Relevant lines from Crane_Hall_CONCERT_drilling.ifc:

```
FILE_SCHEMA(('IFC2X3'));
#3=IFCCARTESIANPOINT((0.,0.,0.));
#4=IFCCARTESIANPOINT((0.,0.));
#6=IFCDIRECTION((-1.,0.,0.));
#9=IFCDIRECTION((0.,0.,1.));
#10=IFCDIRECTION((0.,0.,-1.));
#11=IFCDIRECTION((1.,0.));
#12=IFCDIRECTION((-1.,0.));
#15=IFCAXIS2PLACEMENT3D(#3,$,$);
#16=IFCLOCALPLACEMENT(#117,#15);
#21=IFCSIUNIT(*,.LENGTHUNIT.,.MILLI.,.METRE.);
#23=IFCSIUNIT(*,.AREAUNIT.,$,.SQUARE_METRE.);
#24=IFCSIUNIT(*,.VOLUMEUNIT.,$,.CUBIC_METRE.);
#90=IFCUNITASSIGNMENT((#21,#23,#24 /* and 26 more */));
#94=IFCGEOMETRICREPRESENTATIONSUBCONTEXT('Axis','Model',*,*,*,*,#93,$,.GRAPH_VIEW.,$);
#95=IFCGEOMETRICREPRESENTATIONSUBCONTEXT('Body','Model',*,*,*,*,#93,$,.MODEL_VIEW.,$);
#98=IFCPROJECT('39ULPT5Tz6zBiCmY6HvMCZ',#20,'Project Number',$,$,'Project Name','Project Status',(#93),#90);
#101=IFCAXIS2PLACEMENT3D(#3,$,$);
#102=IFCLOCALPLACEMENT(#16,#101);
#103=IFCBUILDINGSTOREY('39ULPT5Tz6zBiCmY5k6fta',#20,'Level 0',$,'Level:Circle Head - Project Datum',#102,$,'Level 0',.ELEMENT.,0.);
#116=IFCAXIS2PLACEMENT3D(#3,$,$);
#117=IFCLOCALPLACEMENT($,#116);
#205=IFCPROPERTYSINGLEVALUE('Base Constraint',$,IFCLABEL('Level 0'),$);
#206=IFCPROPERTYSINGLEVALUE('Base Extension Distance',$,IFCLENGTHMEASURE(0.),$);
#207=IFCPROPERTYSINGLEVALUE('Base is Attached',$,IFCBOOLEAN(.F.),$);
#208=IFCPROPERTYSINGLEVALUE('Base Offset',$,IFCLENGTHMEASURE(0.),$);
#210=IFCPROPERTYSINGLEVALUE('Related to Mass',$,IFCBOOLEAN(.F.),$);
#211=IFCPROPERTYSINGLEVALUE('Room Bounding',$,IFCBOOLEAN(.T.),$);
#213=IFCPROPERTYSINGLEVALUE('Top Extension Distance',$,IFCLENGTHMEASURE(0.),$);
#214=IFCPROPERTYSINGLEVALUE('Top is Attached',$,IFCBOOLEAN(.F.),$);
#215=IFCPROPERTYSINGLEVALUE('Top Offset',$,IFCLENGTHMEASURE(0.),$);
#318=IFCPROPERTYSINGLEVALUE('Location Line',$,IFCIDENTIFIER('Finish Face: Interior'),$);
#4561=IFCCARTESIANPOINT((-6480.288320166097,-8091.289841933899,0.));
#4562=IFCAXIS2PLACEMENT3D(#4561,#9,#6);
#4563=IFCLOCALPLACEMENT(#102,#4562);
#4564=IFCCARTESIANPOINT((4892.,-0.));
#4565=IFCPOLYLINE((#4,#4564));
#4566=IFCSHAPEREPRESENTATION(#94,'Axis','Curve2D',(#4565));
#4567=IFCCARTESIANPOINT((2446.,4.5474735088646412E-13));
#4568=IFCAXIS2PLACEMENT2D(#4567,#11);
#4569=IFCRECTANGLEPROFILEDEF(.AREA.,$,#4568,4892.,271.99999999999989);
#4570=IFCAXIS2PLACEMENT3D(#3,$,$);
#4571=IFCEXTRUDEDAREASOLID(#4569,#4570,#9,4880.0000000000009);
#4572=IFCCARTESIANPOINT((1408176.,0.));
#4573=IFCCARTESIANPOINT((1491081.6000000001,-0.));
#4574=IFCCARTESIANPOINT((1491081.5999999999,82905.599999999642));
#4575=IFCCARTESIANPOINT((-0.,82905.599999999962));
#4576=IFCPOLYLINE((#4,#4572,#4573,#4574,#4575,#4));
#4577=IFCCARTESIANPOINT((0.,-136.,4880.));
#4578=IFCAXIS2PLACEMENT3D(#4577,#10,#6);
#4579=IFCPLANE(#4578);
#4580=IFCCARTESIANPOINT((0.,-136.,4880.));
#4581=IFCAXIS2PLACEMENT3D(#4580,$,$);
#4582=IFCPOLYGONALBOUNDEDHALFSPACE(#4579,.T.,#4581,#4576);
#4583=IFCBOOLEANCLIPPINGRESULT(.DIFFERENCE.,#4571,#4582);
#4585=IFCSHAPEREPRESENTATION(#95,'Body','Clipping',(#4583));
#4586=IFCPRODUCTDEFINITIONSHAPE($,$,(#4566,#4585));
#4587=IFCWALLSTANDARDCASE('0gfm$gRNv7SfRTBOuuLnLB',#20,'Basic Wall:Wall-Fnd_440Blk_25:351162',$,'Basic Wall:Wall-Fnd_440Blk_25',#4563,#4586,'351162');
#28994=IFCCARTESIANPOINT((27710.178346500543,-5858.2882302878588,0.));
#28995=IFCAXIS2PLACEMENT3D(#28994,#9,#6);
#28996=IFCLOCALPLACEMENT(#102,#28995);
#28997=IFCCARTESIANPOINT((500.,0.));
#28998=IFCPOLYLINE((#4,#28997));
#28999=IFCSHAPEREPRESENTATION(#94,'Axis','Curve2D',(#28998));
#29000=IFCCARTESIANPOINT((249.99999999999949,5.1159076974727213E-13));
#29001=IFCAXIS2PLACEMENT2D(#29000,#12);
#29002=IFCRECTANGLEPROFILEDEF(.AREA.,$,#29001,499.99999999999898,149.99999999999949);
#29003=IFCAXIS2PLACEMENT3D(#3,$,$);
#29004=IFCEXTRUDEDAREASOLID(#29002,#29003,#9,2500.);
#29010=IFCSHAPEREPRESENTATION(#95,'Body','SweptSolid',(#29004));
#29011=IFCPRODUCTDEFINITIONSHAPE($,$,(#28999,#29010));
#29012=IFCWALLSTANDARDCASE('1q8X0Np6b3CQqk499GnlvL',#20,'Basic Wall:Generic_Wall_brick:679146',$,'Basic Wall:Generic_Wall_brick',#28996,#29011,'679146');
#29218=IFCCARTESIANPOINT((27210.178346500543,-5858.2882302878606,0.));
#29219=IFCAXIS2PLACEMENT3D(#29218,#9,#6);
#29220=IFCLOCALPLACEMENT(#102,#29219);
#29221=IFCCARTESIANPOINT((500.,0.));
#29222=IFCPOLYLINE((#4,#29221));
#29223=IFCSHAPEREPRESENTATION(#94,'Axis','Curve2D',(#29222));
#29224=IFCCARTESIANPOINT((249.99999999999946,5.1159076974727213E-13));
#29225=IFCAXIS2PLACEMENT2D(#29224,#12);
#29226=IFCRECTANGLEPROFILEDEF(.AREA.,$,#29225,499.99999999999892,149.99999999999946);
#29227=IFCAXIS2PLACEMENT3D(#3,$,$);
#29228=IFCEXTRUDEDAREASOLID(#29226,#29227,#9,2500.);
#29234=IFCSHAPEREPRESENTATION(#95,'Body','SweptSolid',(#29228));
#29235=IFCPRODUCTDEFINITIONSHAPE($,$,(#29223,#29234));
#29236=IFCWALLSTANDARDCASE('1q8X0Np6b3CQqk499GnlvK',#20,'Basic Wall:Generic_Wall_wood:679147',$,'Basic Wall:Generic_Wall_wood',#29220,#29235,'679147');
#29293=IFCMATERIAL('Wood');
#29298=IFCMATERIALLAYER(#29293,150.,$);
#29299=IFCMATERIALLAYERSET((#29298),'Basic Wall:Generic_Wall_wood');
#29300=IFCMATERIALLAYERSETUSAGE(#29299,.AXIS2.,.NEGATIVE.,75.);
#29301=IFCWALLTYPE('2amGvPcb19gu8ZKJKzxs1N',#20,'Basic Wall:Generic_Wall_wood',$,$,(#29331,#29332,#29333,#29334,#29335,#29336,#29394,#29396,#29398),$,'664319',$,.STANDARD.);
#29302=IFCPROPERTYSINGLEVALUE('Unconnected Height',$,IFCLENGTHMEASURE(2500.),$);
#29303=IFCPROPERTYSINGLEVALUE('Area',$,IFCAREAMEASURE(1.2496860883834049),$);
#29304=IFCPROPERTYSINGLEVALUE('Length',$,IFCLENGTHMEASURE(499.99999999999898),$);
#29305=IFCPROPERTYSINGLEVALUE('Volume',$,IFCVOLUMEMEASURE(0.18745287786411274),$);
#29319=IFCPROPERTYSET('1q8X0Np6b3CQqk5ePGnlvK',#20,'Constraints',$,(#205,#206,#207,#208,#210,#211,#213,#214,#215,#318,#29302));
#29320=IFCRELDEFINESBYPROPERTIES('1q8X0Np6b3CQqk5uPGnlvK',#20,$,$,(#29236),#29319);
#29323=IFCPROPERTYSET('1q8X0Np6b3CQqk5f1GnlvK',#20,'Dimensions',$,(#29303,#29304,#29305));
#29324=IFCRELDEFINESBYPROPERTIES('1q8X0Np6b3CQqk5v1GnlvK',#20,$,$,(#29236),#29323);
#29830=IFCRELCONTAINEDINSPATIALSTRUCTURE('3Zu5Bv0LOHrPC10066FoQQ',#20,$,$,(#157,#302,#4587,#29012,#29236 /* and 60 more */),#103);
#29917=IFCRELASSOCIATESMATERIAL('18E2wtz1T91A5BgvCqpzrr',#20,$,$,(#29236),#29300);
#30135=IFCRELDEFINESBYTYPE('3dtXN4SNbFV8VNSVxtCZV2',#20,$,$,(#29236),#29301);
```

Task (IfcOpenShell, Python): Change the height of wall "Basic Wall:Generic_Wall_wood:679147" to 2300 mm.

```python
import ifcopenshell
import ifcopenshell.api.pset
import ifcopenshell.geom
import ifcopenshell.util.element
import ifcopenshell.util.representation
import ifcopenshell.util.shape
import ifcopenshell.util.unit

model = ifcopenshell.open("Crane_Hall_CONCERT_drilling.ifc")
unit_scale = ifcopenshell.util.unit.calculate_unit_scale(model)
area_scale = ifcopenshell.util.unit.calculate_unit_scale(model, "AREAUNIT")
volume_scale = ifcopenshell.util.unit.calculate_unit_scale(model, "VOLUMEUNIT")
settings = ifcopenshell.geom.settings()


def volume(element):
    """Net volume in cubic metres, openings subtracted."""
    shape = ifcopenshell.geom.create_shape(settings, element)
    return ifcopenshell.util.shape.get_volume(shape.geometry)


wall = model.by_guid("1q8X0Np6b3CQqk499GnlvK")
before = volume(wall)

body = ifcopenshell.util.representation.get_representation(wall, "Model", "Body")
solid = body.Items[0]
old_height = solid.Depth
solid.Depth = 2.3 / unit_scale
after = volume(wall)
thickness = 0.15  # wall thickness in metres

# Update the stored height, areas and volumes.
pset = model.by_id(ifcopenshell.util.element.get_pset(wall, "Constraints", should_inherit=False)["id"])
ifcopenshell.api.pset.edit_pset(model, pset=pset, properties={
    "Unconnected Height": model.create_entity("IfcLengthMeasure", solid.Depth),
})
pset = model.by_id(ifcopenshell.util.element.get_pset(wall, "Dimensions", should_inherit=False)["id"])
ifcopenshell.api.pset.edit_pset(model, pset=pset, properties={
    "Area": model.create_entity("IfcAreaMeasure", after / thickness / area_scale),
    "Volume": model.create_entity("IfcVolumeMeasure", after / volume_scale),
})

print(f"height {old_height:g} -> {solid.Depth:g}, volume {before:.3f} -> {after:.3f} m3")

model.write("Crane_Hall_CONCERT_drilling-out.ifc")
```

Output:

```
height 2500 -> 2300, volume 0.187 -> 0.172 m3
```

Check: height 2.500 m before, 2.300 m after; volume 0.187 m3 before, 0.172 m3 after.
